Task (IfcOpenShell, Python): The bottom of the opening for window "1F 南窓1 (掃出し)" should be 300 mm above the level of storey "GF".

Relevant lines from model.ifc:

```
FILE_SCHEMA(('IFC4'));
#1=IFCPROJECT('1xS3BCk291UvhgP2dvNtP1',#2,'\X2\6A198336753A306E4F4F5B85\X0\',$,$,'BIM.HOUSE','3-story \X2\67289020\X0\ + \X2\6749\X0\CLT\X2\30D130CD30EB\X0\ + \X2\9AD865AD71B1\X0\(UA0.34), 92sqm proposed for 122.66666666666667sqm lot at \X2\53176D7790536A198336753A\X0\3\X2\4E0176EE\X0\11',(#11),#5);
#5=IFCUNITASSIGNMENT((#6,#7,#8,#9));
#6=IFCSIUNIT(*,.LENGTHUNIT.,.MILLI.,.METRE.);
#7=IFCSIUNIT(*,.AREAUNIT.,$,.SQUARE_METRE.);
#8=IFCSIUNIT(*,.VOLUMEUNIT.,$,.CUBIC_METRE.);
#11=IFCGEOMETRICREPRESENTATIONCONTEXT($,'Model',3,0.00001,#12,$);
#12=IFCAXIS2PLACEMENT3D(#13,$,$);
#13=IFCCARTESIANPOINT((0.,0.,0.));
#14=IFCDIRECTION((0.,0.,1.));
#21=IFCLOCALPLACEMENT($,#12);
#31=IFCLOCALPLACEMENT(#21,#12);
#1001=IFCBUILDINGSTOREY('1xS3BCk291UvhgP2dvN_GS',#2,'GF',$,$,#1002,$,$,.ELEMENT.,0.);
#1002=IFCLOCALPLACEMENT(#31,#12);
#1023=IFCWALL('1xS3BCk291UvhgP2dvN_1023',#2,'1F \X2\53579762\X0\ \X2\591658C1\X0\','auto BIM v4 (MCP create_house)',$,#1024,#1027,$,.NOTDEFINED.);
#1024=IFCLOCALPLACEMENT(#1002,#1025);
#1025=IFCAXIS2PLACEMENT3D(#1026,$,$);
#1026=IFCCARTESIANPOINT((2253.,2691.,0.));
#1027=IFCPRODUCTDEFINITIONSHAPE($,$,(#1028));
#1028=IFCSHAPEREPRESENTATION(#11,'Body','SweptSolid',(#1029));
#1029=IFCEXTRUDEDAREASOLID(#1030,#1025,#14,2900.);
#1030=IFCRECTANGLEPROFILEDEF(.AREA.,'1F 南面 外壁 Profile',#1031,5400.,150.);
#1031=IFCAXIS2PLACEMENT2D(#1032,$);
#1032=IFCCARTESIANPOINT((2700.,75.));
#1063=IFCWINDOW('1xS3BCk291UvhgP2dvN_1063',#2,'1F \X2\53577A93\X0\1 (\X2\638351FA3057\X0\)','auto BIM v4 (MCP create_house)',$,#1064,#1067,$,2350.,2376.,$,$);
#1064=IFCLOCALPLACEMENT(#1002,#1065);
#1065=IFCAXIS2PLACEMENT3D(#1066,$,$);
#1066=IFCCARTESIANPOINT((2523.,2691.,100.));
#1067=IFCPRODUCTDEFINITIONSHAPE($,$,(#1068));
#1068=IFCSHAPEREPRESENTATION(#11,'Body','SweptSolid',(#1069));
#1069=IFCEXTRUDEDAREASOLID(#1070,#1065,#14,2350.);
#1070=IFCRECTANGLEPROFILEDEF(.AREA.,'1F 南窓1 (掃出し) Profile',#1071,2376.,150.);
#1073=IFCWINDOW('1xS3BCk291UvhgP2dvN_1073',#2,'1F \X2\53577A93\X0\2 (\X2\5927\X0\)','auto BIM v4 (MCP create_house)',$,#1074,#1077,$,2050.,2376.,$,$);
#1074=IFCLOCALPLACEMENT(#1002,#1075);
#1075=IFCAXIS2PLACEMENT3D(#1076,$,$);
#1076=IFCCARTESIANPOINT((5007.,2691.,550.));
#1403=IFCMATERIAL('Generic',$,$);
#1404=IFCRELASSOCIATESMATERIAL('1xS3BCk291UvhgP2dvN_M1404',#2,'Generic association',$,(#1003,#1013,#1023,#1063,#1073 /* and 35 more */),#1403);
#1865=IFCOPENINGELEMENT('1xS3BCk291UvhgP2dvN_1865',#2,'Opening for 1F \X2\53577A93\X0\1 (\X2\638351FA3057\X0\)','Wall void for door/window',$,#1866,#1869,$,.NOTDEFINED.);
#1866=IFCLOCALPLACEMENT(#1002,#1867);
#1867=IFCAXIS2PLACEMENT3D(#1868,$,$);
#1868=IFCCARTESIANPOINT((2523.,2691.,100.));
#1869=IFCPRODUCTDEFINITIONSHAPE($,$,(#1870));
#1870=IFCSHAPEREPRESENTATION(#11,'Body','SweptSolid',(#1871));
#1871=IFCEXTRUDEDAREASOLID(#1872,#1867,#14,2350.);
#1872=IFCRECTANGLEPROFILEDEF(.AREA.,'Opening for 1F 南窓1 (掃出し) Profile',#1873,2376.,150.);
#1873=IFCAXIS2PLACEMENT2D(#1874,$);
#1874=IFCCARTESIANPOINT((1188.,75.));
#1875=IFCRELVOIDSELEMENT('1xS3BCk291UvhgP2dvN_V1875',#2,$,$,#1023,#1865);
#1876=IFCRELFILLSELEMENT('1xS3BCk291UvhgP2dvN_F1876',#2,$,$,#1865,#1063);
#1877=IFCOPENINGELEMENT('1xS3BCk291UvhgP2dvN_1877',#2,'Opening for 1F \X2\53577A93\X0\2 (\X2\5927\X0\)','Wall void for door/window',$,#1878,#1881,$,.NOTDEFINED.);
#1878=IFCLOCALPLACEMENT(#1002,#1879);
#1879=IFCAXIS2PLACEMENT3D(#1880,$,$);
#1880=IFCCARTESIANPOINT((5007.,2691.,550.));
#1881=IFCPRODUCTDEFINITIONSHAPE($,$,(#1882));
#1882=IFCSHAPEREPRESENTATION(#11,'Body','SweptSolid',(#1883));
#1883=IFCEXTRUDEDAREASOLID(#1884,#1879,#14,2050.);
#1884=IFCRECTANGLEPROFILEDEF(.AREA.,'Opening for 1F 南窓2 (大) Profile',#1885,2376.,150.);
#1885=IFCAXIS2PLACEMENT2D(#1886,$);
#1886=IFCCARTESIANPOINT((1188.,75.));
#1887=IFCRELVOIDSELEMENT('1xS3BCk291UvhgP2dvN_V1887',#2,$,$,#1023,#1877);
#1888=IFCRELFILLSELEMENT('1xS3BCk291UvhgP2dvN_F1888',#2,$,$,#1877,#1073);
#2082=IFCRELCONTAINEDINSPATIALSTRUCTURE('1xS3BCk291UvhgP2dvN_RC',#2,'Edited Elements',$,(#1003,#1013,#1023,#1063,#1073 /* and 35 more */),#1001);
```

```python
import numpy as np
import ifcopenshell
import ifcopenshell.api.geometry
import ifcopenshell.geom
import ifcopenshell.util.element
import ifcopenshell.util.placement
import ifcopenshell.util.shape
import ifcopenshell.util.unit

model = ifcopenshell.open("model.ifc")
unit_scale = ifcopenshell.util.unit.calculate_unit_scale(model)

window = model.by_id(1063)
opening = window.FillsVoids[0].RelatingOpeningElement
storey = ifcopenshell.util.element.get_container(window, ifc_class="IfcBuildingStorey")
level = ifcopenshell.util.placement.get_local_placement(storey.ObjectPlacement)[2, 3]

# The opening's origin need not be at the sill, so measure its lowest point.
shape = ifcopenshell.geom.create_shape(ifcopenshell.geom.settings(), opening)
bottom = ifcopenshell.util.shape.get_shape_bottom_elevation(shape, shape.geometry) / unit_scale
dz = level + 300.0 - bottom

shift = np.array([0.0, 0.0, dz])
# The window is not placed relative to its opening, so move both.
for product in (opening, window):
    matrix = ifcopenshell.util.placement.get_local_placement(product.ObjectPlacement)
    matrix[:3, 3] += shift
    ifcopenshell.api.geometry.edit_object_placement(model, product=product, matrix=matrix, is_si=False)

print(f"moved by {dz * unit_scale:+.3f} m")

model.write("model_updated.ifc")
```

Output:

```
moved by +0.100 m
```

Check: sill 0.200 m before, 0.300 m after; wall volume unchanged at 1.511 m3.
